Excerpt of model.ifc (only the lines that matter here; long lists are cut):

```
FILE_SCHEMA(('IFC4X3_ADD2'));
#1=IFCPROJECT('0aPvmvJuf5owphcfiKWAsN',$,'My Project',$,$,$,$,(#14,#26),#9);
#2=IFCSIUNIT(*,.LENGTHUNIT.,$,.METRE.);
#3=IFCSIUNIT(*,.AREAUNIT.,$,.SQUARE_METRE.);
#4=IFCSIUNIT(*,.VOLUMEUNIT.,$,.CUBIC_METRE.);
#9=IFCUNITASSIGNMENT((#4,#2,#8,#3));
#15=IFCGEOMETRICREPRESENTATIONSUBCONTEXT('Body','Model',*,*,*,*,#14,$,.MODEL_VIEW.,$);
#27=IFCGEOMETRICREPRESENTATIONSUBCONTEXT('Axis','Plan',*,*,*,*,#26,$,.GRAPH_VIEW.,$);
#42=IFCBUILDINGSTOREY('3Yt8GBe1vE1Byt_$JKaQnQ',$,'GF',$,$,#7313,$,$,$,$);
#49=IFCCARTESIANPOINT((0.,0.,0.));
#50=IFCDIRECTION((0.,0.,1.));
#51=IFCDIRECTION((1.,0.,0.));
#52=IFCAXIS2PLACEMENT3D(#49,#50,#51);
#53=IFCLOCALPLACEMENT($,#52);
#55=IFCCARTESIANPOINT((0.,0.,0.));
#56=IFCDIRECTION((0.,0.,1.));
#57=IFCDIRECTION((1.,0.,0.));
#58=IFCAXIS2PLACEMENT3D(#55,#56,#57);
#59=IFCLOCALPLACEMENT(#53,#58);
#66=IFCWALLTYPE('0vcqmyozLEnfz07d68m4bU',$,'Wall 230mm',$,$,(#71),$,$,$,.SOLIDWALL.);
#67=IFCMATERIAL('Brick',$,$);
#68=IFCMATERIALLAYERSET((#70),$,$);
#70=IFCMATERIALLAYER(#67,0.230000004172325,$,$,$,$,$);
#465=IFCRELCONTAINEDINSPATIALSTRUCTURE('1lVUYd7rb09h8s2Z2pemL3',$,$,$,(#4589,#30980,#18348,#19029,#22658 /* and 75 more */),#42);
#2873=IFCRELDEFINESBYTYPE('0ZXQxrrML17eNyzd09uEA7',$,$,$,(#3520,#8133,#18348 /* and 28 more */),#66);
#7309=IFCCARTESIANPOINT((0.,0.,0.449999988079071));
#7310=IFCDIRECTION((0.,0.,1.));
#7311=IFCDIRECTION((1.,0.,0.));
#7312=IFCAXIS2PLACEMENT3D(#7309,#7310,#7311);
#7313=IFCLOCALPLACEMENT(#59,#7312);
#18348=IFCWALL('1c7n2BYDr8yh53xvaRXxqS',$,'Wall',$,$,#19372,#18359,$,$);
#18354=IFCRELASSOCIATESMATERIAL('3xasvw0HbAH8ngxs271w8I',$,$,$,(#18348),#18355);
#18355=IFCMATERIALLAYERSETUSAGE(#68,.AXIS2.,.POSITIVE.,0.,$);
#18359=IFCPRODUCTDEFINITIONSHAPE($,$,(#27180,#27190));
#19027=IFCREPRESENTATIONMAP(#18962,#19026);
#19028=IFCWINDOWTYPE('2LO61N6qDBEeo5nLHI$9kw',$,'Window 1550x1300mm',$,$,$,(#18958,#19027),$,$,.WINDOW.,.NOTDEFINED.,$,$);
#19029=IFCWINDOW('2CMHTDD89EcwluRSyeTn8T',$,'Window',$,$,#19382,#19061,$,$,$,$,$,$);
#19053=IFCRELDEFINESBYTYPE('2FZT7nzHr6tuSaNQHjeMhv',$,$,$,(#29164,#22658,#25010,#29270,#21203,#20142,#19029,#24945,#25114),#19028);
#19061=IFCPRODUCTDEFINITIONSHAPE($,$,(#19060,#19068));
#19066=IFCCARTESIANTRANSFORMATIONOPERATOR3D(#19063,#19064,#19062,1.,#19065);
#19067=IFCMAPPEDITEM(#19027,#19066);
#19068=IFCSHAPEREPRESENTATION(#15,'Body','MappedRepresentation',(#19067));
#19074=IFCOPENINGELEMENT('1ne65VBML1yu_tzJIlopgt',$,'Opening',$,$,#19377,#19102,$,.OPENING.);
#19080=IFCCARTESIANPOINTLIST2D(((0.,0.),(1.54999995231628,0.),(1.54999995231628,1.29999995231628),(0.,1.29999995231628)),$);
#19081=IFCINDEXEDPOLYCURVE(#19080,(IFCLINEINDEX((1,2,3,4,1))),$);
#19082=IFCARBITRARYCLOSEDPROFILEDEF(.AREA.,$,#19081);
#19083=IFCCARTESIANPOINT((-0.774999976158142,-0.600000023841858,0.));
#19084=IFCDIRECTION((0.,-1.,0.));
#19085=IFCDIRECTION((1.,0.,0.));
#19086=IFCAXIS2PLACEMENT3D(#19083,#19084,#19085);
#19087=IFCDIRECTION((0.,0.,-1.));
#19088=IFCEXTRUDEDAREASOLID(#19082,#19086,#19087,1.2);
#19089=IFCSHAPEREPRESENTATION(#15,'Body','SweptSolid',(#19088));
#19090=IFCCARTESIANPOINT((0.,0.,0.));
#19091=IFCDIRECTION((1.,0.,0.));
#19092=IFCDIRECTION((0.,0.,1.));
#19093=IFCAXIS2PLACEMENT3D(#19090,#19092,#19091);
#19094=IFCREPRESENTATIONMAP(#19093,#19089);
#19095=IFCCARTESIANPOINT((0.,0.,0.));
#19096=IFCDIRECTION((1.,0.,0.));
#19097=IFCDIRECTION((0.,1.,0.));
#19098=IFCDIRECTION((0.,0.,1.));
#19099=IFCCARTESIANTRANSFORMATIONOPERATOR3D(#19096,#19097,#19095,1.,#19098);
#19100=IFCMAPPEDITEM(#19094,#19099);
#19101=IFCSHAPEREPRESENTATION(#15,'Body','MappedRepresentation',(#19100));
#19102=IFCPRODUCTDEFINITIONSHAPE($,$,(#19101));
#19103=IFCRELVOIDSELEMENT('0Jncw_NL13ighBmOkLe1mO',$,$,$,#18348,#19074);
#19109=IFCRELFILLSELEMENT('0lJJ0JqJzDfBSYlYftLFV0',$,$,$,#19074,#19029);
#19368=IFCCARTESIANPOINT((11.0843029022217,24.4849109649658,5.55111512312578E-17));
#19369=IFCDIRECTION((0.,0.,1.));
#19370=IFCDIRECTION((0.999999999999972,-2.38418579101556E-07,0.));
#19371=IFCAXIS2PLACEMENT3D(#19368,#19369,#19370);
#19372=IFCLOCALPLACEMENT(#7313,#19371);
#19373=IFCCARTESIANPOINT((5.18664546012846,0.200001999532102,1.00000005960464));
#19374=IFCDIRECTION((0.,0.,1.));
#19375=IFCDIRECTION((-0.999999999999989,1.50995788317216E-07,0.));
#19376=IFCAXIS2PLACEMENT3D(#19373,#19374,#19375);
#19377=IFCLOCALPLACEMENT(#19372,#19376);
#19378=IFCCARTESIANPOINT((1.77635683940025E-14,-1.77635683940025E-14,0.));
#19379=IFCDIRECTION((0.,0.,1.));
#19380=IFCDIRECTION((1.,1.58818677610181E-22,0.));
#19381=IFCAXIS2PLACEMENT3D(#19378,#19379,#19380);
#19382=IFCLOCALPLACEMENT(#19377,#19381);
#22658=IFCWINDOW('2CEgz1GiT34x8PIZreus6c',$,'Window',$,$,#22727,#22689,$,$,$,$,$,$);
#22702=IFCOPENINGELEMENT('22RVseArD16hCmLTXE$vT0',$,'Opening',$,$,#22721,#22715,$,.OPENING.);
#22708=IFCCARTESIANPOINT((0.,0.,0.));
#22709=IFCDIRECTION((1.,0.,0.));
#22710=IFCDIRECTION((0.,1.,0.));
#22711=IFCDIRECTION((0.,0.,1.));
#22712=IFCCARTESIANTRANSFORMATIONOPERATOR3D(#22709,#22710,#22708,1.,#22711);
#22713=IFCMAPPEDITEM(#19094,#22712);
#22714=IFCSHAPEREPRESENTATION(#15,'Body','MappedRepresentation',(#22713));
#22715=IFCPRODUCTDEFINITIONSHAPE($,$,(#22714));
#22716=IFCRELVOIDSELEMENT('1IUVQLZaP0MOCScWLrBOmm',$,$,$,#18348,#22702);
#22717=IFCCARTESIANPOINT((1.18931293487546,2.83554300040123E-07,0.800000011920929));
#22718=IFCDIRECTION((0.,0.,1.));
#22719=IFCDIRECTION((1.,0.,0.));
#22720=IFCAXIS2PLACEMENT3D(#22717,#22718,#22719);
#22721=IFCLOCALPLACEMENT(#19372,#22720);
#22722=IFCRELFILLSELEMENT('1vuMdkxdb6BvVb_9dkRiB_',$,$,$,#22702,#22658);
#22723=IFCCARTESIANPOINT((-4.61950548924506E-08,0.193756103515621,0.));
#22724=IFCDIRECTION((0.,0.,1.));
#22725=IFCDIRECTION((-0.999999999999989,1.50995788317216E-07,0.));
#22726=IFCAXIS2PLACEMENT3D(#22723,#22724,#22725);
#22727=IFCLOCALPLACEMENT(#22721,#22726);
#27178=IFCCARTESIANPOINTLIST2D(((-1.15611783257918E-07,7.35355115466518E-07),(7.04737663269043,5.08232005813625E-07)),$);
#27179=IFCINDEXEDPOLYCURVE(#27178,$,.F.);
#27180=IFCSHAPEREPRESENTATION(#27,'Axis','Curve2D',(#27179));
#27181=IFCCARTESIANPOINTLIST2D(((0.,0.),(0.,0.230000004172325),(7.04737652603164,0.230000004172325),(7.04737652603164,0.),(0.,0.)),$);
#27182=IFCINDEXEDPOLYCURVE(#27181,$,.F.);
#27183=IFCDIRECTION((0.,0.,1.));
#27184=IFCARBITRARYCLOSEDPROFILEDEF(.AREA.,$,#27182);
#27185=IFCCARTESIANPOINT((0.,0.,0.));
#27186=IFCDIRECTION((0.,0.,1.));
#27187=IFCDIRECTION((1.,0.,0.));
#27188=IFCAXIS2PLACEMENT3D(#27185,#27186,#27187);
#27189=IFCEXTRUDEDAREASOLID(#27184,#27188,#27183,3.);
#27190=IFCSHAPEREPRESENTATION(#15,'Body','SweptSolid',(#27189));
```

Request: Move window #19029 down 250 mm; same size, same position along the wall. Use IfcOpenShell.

```python
import numpy as np
import ifcopenshell
import ifcopenshell.api.geometry
import ifcopenshell.util.placement
import ifcopenshell.util.unit

model = ifcopenshell.open("model.ifc")
unit_scale = ifcopenshell.util.unit.calculate_unit_scale(model)

window = model.by_id(19029)
opening = window.FillsVoids[0].RelatingOpeningElement
dz = -0.25

shift = np.array([0.0, 0.0, dz])
# The window is placed relative to its opening, so it follows when the opening moves.
matrix = ifcopenshell.util.placement.get_local_placement(opening.ObjectPlacement)
matrix[:3, 3] += shift
ifcopenshell.api.geometry.edit_object_placement(
    model, product=opening, matrix=matrix, is_si=False, should_transform_children=True
)

print(f"moved by {dz * unit_scale:+.3f} m")

model.write("model_rev.ifc")
```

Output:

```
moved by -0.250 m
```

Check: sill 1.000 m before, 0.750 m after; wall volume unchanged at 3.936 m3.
